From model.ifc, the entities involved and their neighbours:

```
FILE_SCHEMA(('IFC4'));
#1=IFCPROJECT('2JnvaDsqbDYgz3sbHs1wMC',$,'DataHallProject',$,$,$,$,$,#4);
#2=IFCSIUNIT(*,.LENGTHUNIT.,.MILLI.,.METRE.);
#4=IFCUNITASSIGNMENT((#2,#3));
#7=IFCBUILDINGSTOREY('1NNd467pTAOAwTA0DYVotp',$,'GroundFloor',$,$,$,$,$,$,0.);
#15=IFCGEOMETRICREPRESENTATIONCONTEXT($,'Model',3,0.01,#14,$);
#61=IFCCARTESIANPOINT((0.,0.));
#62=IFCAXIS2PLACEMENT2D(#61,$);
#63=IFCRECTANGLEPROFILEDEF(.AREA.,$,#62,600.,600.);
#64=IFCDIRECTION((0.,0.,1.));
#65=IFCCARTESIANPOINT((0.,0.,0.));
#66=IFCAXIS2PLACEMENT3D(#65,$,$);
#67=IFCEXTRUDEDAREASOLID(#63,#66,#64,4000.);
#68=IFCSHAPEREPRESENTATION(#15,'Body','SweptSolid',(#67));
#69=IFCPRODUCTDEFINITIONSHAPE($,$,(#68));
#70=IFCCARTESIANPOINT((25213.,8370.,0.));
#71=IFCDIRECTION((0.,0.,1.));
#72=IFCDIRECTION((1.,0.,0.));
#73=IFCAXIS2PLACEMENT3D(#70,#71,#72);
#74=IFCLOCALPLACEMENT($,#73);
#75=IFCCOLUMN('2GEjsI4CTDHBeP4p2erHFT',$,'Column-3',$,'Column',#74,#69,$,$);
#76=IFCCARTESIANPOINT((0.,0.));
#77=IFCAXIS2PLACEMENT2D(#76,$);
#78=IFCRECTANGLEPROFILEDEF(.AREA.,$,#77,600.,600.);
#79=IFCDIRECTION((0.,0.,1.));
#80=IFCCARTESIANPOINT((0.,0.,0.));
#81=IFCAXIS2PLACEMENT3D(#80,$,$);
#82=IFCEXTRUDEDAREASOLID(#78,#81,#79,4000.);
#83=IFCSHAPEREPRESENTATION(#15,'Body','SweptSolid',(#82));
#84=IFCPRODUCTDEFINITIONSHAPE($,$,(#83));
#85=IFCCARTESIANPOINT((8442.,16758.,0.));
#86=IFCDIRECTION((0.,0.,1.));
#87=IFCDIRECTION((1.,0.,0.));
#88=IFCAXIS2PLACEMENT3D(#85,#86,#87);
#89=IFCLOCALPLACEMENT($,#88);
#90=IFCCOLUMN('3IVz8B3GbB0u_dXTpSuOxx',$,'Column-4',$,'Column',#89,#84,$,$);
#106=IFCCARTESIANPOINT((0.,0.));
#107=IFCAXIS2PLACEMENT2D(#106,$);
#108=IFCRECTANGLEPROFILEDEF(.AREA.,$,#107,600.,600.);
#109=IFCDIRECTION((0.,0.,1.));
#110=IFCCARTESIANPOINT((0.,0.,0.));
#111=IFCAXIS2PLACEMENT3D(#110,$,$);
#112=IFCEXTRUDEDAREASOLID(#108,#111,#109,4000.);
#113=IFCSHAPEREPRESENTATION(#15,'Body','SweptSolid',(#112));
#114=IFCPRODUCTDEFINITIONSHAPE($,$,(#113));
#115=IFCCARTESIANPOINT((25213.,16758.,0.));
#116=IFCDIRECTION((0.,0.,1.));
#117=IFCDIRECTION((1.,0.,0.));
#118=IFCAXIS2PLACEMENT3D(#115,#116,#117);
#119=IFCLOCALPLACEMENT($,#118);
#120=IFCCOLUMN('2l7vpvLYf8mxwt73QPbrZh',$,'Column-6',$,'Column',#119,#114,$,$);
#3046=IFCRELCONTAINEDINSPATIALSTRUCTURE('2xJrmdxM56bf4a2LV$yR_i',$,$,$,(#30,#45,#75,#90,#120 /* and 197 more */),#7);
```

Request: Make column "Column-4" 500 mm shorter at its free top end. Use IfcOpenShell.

```python
import ifcopenshell

model = ifcopenshell.open("model.ifc")

member = model.by_guid("3IVz8B3GbB0u_dXTpSuOxx")
change = -500.0

# The extrusion runs towards the end named, so only its depth changes.
body = next(r for r in member.Representation.Representations if r.RepresentationIdentifier == "Body")
solid = body.Items[0]
old_length = solid.Depth
solid.Depth += change

print(f"length {old_length:g} -> {solid.Depth:g}")

model.write("model-out.ifc")
```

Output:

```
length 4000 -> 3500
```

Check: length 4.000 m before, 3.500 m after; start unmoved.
